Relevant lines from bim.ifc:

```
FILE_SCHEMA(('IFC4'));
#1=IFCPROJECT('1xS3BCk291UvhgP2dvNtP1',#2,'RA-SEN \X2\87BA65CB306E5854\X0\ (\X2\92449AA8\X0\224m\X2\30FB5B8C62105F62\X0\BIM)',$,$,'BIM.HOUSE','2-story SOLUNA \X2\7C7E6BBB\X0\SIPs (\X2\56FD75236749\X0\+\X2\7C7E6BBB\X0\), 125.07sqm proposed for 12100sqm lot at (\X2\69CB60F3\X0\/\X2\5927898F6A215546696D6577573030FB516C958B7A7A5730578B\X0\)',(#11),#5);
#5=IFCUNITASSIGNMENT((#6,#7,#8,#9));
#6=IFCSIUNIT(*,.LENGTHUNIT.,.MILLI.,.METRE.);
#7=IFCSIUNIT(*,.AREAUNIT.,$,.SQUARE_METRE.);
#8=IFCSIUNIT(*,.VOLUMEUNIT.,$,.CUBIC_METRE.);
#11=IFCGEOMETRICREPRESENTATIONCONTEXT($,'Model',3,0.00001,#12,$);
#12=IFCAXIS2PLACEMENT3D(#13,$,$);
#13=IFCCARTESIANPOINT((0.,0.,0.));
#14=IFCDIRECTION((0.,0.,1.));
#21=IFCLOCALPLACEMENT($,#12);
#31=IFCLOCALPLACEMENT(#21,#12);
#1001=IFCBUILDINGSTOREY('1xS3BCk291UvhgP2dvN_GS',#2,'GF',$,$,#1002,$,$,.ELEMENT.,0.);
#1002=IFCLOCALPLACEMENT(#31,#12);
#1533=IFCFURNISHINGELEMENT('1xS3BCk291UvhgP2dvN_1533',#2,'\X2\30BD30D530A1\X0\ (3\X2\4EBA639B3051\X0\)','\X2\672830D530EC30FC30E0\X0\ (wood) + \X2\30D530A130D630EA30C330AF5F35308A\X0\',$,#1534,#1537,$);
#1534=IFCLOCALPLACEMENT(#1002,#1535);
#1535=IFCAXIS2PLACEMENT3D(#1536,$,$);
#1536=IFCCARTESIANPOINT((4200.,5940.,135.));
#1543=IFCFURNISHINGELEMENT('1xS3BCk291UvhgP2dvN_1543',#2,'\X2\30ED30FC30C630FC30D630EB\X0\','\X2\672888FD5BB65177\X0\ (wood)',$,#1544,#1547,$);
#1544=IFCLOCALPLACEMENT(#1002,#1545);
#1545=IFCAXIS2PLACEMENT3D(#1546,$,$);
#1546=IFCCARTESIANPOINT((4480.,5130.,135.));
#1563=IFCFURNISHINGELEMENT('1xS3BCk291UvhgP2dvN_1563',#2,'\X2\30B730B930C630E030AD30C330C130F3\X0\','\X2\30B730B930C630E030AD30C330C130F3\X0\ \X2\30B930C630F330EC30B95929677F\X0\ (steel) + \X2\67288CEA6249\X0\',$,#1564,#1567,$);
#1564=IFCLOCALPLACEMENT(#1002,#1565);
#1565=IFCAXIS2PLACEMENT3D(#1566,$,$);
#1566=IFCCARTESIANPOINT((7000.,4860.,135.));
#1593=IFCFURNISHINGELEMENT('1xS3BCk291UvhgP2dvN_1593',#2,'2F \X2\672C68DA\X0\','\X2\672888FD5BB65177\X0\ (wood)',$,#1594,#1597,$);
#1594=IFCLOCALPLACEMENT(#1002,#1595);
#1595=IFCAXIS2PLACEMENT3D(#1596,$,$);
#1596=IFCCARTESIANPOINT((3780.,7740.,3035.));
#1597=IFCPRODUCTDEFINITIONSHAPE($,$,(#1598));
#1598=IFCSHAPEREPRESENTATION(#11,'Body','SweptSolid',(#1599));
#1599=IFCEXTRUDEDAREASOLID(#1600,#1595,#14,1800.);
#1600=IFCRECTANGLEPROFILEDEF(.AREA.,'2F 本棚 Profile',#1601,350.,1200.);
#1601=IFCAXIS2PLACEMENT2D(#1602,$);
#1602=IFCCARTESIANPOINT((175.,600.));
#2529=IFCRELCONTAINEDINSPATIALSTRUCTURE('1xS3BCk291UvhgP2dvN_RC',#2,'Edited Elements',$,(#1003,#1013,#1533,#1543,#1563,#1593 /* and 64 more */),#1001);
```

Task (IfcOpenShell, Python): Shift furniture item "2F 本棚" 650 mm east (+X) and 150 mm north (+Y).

```python
import ifcopenshell
import ifcopenshell.api.geometry
import ifcopenshell.util.placement
import ifcopenshell.util.unit

model = ifcopenshell.open("bim.ifc")
unit_scale = ifcopenshell.util.unit.calculate_unit_scale(model)

item = model.by_guid("1xS3BCk291UvhgP2dvN_1593")
matrix = ifcopenshell.util.placement.get_local_placement(item.ObjectPlacement)
matrix[0, 3] += 0.65 / unit_scale
matrix[1, 3] += 0.15 / unit_scale
ifcopenshell.api.geometry.edit_object_placement(model, product=item, matrix=matrix, is_si=False)

print(ifcopenshell.util.placement.get_local_placement(item.ObjectPlacement).round(3) + 0.0)

model.write("bim_updated.ifc")
```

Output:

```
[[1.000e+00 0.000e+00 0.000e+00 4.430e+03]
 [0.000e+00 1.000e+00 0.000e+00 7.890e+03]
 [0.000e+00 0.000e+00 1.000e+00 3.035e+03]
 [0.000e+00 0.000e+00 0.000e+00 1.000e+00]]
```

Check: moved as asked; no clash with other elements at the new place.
